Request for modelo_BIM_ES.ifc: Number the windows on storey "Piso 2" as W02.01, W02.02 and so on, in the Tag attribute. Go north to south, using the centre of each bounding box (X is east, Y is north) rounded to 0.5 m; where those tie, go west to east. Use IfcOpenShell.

First a look at what the model holds.

```python
import ifcopenshell
import ifcopenshell.util.element
import ifcopenshell.util.placement

model = ifcopenshell.open("modelo_BIM_ES.ifc")
print(model.schema)
storey = next(s for s in model.by_type("IfcBuildingStorey") if s.Name == "Piso 2")
windows = [e for e in ifcopenshell.util.element.get_decomposition(storey) if e.is_a("IfcWindow")]
for e in sorted(windows, key=lambda e: e.id()):
    origin = ifcopenshell.util.placement.get_local_placement(e.ObjectPlacement)[:3, 3]
    print(e.id(), e.Tag, e.Name, origin.round(2) + 0.0, sep=" | ")
```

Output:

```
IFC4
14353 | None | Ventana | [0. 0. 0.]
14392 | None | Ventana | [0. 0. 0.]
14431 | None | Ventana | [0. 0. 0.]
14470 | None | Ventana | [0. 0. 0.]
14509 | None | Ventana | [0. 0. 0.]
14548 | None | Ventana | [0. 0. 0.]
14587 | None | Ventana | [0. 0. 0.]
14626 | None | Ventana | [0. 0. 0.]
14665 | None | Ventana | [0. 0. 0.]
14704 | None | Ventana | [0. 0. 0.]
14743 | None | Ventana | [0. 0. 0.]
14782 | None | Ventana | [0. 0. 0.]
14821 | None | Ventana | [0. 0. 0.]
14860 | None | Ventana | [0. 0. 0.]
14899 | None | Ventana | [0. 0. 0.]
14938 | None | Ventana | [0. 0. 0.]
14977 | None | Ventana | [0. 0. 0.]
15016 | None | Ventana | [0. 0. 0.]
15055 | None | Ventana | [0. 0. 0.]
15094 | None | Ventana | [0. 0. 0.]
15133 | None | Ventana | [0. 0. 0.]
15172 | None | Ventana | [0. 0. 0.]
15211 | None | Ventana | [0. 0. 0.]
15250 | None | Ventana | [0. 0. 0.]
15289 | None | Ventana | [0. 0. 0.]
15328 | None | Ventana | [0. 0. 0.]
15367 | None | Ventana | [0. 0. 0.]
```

```python
import ifcopenshell
import ifcopenshell.geom
import ifcopenshell.util.element
import ifcopenshell.util.shape

model = ifcopenshell.open("modelo_BIM_ES.ifc")
settings = ifcopenshell.geom.settings()
settings.set("use-world-coords", True)


def centre(element):
    shape = ifcopenshell.geom.create_shape(settings, element)
    return ifcopenshell.util.shape.get_bbox_centroid(shape.geometry)


storey = next(s for s in model.by_type("IfcBuildingStorey") if s.Name == "Piso 2")
windows = [e for e in ifcopenshell.util.element.get_decomposition(storey) if e.is_a("IfcWindow")]

# Insertion points can sit at a corner or the storey origin, so sort by the geometry (in metres).
centres = {e: centre(e) for e in windows}
windows.sort(key=lambda e: (-round(centres[e][1] / 0.5), centres[e][0]))

for i, e in enumerate(windows, start=1):
    number = f"W02.{i:02d}"
    e.Tag = number
    print(e.id(), number)

model.write("modelo_BIM_ES_updated.ifc")
```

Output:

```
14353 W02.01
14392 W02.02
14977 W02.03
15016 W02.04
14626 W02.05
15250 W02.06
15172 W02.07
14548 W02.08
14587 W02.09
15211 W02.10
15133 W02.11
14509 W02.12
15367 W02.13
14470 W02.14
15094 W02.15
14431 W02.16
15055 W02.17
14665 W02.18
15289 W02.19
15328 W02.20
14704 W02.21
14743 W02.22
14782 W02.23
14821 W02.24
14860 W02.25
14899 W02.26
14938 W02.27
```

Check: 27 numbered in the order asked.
